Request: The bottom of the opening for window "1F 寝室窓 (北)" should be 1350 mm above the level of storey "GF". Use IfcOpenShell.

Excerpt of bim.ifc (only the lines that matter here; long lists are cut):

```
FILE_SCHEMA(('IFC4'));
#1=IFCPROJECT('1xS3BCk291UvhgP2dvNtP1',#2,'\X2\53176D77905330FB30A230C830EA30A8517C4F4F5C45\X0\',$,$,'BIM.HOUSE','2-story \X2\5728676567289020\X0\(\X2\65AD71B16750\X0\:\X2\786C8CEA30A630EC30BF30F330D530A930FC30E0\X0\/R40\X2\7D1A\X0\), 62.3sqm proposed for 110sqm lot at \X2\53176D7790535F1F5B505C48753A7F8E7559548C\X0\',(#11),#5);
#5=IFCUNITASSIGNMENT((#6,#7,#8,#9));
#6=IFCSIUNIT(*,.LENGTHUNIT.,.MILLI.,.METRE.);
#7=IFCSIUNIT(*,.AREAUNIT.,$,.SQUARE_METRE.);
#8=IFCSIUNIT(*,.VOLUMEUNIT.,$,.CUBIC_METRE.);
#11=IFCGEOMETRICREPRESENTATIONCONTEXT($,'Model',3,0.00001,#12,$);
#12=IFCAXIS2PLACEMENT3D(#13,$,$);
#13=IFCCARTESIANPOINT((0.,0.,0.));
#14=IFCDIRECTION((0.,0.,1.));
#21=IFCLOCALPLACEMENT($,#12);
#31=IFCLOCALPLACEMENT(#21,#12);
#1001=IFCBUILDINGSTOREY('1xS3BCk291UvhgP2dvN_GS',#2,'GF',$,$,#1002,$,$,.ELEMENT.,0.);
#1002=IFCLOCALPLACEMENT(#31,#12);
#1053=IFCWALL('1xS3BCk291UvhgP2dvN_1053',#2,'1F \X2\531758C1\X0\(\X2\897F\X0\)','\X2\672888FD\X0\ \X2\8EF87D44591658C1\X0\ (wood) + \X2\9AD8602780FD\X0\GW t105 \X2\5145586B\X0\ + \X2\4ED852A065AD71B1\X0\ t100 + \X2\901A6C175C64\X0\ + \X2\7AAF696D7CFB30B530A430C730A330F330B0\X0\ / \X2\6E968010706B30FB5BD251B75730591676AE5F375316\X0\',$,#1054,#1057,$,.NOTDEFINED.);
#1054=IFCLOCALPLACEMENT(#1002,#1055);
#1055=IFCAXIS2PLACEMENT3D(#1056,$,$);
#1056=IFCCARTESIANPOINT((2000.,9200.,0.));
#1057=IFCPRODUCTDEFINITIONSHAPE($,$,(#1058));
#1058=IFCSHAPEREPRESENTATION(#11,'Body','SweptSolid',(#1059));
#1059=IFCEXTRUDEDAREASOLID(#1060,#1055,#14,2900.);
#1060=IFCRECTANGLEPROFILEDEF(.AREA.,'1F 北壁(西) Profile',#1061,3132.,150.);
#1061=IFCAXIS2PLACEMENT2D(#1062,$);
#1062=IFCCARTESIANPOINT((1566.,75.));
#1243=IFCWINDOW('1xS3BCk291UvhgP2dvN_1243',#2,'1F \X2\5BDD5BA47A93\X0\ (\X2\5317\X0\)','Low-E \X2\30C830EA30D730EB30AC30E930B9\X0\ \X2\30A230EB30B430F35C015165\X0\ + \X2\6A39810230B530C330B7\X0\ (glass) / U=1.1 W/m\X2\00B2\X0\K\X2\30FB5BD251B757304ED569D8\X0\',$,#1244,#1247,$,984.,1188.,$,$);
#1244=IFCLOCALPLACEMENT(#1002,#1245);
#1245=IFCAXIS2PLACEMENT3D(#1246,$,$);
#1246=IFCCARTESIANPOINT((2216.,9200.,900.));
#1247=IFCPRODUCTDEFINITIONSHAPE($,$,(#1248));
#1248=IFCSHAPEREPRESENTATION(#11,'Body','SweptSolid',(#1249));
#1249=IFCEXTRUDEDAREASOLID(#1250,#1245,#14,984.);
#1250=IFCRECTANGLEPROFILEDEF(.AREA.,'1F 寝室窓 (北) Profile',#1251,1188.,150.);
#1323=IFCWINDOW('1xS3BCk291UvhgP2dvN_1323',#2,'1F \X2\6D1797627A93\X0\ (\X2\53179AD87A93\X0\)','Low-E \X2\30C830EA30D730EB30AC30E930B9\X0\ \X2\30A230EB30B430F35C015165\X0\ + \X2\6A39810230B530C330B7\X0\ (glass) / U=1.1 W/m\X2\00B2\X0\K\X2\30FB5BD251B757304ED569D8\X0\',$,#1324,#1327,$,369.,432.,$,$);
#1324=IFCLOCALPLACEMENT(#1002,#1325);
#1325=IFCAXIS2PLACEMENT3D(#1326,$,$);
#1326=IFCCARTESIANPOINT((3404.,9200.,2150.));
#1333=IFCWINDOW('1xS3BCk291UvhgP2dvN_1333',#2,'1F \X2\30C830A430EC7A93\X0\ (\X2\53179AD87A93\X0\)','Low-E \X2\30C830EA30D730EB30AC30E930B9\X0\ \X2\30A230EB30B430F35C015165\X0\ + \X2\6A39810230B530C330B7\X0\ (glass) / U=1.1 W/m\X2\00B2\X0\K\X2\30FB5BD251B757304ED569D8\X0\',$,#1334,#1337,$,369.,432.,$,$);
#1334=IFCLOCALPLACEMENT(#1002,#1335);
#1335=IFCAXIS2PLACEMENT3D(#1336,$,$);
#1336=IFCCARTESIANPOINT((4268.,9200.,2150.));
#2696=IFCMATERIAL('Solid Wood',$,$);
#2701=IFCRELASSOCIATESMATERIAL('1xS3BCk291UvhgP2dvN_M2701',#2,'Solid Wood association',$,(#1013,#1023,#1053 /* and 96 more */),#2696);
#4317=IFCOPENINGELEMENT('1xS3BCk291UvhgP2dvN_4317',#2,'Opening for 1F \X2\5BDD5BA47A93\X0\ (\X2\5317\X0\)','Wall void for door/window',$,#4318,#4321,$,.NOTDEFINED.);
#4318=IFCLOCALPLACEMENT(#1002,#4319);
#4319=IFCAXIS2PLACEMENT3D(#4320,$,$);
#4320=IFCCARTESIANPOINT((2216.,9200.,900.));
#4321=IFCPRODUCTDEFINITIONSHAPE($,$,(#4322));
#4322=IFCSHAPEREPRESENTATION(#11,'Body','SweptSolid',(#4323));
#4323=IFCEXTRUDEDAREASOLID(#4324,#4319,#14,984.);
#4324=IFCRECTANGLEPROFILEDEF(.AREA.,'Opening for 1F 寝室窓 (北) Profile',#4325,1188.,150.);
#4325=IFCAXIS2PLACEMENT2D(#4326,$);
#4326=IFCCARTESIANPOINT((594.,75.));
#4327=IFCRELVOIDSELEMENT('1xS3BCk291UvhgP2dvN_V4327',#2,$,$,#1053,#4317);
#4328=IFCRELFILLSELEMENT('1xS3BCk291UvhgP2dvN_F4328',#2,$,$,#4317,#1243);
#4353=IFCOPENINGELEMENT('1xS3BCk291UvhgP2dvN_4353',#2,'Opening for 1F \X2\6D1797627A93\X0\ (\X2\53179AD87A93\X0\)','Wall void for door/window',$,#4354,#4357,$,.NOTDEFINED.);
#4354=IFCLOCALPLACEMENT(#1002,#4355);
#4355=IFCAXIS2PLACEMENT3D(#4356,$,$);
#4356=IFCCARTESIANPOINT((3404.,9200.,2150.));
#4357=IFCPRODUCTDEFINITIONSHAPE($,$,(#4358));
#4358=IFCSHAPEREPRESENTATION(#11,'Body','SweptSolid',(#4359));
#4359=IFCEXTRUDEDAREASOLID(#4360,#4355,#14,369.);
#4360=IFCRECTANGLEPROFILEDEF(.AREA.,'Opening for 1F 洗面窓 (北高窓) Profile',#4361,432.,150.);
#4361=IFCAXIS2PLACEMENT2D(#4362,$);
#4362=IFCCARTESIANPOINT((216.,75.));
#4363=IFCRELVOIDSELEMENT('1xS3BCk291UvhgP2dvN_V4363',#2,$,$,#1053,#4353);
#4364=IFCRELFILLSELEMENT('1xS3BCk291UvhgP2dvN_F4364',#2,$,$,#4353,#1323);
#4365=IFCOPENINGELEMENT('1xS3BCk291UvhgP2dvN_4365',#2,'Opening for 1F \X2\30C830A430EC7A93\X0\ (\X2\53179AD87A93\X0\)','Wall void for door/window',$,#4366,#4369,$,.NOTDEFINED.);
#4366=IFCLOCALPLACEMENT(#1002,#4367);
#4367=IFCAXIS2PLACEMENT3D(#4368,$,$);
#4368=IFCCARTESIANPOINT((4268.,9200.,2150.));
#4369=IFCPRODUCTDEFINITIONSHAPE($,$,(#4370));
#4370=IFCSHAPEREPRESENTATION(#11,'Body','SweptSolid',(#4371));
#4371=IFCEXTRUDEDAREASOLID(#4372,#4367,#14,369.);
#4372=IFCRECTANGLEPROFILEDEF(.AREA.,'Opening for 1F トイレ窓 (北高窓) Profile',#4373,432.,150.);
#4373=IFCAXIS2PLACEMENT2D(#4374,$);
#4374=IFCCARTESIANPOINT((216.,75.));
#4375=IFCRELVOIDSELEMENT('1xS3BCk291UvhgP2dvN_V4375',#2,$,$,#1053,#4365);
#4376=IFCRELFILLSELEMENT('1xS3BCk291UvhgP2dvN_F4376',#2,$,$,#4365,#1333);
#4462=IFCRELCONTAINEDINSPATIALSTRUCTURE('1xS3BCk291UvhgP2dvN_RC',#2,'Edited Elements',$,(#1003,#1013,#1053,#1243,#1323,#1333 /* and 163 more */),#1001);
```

```python
import numpy as np
import ifcopenshell
import ifcopenshell.api.geometry
import ifcopenshell.geom
import ifcopenshell.util.element
import ifcopenshell.util.placement
import ifcopenshell.util.shape
import ifcopenshell.util.unit

model = ifcopenshell.open("bim.ifc")
unit_scale = ifcopenshell.util.unit.calculate_unit_scale(model)

window = model.by_guid("1xS3BCk291UvhgP2dvN_1243")
opening = window.FillsVoids[0].RelatingOpeningElement
storey = ifcopenshell.util.element.get_container(window, ifc_class="IfcBuildingStorey")
level = ifcopenshell.util.placement.get_local_placement(storey.ObjectPlacement)[2, 3]

# The opening's origin need not be at the sill, so measure its lowest point.
shape = ifcopenshell.geom.create_shape(ifcopenshell.geom.settings(), opening)
bottom = ifcopenshell.util.shape.get_shape_bottom_elevation(shape, shape.geometry) / unit_scale
dz = level + 1.35 / unit_scale - bottom

shift = np.array([0.0, 0.0, dz])
# The window is not placed relative to its opening, so move both.
for product in (opening, window):
    matrix = ifcopenshell.util.placement.get_local_placement(product.ObjectPlacement)
    matrix[:3, 3] += shift
    ifcopenshell.api.geometry.edit_object_placement(model, product=product, matrix=matrix, is_si=False)

print(f"moved by {dz * unit_scale:+.3f} m")

model.write("bim_rev.ifc")
```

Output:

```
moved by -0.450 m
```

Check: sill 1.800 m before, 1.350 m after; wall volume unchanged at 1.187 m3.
